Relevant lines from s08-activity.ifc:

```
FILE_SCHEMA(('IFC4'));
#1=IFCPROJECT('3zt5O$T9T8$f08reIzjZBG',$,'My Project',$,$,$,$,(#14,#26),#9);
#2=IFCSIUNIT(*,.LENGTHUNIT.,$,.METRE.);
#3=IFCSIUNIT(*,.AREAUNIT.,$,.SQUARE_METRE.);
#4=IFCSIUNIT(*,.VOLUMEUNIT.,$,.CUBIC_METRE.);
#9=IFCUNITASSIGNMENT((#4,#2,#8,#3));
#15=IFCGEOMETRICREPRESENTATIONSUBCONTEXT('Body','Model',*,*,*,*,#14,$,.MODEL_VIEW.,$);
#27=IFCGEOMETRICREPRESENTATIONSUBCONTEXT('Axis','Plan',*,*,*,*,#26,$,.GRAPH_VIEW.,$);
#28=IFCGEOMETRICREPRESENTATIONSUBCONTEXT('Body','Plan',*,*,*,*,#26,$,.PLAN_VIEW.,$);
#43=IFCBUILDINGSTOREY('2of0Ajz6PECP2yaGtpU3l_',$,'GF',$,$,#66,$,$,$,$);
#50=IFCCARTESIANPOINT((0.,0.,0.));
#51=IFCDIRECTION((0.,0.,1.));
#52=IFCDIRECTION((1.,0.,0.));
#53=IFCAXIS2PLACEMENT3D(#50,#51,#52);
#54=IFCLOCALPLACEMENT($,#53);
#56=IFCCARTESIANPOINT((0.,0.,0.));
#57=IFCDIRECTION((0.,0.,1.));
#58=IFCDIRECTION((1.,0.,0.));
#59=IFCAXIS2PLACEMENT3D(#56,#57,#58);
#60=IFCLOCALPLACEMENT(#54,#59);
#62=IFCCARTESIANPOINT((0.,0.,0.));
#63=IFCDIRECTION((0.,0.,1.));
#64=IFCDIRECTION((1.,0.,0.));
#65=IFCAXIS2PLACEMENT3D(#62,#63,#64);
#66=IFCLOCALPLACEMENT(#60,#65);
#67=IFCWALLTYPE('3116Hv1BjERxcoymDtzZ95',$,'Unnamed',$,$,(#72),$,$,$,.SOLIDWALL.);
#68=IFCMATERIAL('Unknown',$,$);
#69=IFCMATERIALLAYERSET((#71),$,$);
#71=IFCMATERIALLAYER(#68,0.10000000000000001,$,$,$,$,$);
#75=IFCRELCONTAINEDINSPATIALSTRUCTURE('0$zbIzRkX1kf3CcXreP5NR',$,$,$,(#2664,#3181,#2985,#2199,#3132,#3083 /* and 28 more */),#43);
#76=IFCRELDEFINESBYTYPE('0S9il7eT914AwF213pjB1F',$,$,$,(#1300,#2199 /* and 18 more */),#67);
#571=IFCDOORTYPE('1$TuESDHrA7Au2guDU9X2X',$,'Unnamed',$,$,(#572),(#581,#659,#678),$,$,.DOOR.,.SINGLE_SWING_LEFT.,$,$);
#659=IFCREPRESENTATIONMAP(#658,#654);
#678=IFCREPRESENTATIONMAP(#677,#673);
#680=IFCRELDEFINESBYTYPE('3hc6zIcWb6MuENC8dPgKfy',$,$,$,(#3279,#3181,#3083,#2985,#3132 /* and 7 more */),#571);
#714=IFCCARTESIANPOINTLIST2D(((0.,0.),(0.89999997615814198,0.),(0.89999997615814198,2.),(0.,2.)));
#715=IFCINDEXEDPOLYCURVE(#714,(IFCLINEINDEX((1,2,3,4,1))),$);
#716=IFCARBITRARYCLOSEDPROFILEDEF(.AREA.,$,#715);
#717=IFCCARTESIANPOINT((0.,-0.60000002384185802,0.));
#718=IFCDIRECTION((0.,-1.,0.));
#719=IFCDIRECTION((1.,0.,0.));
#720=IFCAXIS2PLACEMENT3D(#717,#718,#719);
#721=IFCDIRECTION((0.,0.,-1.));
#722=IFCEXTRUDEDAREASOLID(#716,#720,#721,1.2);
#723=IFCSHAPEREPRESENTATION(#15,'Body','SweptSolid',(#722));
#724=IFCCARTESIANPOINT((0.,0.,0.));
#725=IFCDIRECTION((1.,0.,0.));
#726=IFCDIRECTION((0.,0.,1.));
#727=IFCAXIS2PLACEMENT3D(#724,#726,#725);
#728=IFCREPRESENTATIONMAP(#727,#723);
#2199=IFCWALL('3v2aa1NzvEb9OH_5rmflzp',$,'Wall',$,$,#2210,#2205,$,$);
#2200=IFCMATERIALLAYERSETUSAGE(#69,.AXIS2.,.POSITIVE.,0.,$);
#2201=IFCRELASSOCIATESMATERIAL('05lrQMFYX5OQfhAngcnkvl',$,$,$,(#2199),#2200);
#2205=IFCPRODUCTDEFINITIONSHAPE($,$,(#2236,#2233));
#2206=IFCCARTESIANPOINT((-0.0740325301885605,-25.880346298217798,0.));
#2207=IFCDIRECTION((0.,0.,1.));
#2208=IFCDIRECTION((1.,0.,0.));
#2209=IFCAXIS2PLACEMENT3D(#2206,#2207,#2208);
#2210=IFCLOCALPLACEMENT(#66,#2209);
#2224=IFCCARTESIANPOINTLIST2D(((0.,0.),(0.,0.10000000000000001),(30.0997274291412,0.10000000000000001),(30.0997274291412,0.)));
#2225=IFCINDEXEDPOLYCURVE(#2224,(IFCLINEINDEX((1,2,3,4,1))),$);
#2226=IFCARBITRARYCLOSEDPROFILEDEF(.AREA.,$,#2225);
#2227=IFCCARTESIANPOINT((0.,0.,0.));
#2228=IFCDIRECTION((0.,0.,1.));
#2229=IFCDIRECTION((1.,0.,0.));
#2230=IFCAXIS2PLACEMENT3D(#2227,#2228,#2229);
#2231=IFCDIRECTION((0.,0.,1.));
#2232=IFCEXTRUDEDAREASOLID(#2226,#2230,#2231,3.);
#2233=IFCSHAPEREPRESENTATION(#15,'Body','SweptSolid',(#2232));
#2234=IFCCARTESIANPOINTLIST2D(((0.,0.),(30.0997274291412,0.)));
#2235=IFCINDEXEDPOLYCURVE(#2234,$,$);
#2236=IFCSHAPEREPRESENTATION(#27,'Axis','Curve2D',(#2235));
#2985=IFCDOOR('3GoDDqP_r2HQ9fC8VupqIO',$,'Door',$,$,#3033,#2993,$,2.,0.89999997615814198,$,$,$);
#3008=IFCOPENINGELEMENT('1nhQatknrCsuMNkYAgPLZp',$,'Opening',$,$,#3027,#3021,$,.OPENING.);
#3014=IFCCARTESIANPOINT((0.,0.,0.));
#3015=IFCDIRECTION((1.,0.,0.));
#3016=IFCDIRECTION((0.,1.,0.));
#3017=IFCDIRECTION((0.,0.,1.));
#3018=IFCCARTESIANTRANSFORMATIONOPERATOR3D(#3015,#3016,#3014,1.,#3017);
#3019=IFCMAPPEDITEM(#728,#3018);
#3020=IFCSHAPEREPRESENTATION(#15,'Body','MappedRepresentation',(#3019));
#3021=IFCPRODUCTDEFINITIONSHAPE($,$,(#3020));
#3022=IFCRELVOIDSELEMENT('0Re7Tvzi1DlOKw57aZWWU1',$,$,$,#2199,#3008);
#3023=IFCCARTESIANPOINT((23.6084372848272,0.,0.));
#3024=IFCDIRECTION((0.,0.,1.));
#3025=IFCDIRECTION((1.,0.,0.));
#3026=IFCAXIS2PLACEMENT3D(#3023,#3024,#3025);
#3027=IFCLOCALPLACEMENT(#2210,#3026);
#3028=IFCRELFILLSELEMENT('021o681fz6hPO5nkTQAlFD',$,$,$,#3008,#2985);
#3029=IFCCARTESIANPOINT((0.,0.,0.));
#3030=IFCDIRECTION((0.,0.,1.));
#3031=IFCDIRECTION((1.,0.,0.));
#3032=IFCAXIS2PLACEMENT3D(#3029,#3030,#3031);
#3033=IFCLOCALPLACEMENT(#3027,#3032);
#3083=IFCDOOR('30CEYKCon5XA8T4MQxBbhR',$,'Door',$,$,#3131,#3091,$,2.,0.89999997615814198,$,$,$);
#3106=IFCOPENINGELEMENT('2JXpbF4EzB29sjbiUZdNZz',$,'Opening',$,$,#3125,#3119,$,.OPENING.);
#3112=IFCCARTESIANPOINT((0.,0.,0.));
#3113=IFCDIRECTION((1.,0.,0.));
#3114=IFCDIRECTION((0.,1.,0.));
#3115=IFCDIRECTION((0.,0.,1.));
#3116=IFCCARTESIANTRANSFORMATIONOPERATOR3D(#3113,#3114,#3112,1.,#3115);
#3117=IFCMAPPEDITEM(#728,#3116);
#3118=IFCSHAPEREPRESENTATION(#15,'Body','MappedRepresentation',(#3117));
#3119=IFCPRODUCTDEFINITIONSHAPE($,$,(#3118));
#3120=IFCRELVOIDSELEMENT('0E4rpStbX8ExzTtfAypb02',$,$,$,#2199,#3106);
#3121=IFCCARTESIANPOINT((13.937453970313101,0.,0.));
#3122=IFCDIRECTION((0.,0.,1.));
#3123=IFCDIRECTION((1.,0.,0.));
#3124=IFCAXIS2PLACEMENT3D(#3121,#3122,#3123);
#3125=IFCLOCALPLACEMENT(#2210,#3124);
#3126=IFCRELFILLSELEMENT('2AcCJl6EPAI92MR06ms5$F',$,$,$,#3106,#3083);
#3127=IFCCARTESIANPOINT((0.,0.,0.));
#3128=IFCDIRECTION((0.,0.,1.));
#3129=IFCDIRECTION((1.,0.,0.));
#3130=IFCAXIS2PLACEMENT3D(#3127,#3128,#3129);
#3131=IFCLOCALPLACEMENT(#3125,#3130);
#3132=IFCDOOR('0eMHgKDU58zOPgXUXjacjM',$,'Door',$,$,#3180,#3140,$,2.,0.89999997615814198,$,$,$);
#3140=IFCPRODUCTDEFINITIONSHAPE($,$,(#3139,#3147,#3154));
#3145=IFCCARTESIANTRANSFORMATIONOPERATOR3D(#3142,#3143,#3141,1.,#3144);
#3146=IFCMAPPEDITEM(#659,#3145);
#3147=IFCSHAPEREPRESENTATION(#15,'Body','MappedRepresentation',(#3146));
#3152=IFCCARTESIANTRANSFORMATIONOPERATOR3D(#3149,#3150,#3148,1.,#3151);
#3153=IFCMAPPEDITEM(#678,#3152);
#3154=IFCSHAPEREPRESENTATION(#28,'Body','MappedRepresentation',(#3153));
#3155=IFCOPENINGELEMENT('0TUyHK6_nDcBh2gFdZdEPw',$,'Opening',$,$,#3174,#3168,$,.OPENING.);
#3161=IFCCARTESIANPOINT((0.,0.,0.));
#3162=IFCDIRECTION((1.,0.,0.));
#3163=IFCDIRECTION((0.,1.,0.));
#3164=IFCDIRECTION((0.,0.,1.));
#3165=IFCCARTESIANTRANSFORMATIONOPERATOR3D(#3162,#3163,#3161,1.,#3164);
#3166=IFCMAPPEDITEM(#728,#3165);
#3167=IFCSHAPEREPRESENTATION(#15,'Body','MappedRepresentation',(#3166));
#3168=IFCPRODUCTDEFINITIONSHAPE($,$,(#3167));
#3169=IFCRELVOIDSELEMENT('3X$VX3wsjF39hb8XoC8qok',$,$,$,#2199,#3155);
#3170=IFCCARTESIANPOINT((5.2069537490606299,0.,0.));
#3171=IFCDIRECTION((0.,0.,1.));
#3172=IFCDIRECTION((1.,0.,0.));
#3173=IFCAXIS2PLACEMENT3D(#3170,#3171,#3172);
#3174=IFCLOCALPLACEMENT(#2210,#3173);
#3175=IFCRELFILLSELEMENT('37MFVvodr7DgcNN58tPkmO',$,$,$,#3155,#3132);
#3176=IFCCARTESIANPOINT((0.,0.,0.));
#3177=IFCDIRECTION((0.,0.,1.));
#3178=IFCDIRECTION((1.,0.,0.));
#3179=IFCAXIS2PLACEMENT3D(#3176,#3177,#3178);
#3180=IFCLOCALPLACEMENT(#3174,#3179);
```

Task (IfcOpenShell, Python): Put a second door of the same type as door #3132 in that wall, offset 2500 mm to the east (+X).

```python
import ifcopenshell
import ifcopenshell.api.feature
import ifcopenshell.api.geometry
import ifcopenshell.api.root
import ifcopenshell.geom
import ifcopenshell.util.element
import ifcopenshell.util.placement
import ifcopenshell.util.shape
import ifcopenshell.util.unit

model = ifcopenshell.open("s08-activity.ifc")
unit_scale = ifcopenshell.util.unit.calculate_unit_scale(model)
settings = ifcopenshell.geom.settings()


def volume(element):
    """Net volume in cubic metres, openings subtracted."""
    shape = ifcopenshell.geom.create_shape(settings, element)
    return ifcopenshell.util.shape.get_volume(shape.geometry)


door = model.by_id(3132)
opening = door.FillsVoids[0].RelatingOpeningElement
wall = opening.VoidsElements[0].RelatingBuildingElement
before = volume(wall)
shift = ifcopenshell.util.placement.get_local_placement(wall.ObjectPlacement)[:3, 0] * 2.5 / unit_scale

# copy_class copies the void relationship, type, container and properties, but no geometry.
new_opening = ifcopenshell.api.root.copy_class(model, product=opening)
new_opening.Representation = ifcopenshell.util.element.copy_deep(
    model, opening.Representation, exclude=["IfcGeometricRepresentationContext", "IfcRepresentationMap"]
)
new_door = ifcopenshell.api.root.copy_class(model, product=door)
new_door.Representation = ifcopenshell.util.element.copy_deep(
    model, door.Representation, exclude=["IfcGeometricRepresentationContext", "IfcRepresentationMap"]
)
ifcopenshell.api.feature.add_filling(model, opening=new_opening, element=new_door)

for old, new in ((opening, new_opening), (door, new_door)):
    matrix = ifcopenshell.util.placement.get_local_placement(old.ObjectPlacement)
    matrix[:3, 3] += shift
    ifcopenshell.api.geometry.edit_object_placement(model, product=new, matrix=matrix, is_si=False)

after = volume(wall)

print(f"wall volume {before:.3f} -> {after:.3f} m3")

model.write("s08-activity-out.ifc")
```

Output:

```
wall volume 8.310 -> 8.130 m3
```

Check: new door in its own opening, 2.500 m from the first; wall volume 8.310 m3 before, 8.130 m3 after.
